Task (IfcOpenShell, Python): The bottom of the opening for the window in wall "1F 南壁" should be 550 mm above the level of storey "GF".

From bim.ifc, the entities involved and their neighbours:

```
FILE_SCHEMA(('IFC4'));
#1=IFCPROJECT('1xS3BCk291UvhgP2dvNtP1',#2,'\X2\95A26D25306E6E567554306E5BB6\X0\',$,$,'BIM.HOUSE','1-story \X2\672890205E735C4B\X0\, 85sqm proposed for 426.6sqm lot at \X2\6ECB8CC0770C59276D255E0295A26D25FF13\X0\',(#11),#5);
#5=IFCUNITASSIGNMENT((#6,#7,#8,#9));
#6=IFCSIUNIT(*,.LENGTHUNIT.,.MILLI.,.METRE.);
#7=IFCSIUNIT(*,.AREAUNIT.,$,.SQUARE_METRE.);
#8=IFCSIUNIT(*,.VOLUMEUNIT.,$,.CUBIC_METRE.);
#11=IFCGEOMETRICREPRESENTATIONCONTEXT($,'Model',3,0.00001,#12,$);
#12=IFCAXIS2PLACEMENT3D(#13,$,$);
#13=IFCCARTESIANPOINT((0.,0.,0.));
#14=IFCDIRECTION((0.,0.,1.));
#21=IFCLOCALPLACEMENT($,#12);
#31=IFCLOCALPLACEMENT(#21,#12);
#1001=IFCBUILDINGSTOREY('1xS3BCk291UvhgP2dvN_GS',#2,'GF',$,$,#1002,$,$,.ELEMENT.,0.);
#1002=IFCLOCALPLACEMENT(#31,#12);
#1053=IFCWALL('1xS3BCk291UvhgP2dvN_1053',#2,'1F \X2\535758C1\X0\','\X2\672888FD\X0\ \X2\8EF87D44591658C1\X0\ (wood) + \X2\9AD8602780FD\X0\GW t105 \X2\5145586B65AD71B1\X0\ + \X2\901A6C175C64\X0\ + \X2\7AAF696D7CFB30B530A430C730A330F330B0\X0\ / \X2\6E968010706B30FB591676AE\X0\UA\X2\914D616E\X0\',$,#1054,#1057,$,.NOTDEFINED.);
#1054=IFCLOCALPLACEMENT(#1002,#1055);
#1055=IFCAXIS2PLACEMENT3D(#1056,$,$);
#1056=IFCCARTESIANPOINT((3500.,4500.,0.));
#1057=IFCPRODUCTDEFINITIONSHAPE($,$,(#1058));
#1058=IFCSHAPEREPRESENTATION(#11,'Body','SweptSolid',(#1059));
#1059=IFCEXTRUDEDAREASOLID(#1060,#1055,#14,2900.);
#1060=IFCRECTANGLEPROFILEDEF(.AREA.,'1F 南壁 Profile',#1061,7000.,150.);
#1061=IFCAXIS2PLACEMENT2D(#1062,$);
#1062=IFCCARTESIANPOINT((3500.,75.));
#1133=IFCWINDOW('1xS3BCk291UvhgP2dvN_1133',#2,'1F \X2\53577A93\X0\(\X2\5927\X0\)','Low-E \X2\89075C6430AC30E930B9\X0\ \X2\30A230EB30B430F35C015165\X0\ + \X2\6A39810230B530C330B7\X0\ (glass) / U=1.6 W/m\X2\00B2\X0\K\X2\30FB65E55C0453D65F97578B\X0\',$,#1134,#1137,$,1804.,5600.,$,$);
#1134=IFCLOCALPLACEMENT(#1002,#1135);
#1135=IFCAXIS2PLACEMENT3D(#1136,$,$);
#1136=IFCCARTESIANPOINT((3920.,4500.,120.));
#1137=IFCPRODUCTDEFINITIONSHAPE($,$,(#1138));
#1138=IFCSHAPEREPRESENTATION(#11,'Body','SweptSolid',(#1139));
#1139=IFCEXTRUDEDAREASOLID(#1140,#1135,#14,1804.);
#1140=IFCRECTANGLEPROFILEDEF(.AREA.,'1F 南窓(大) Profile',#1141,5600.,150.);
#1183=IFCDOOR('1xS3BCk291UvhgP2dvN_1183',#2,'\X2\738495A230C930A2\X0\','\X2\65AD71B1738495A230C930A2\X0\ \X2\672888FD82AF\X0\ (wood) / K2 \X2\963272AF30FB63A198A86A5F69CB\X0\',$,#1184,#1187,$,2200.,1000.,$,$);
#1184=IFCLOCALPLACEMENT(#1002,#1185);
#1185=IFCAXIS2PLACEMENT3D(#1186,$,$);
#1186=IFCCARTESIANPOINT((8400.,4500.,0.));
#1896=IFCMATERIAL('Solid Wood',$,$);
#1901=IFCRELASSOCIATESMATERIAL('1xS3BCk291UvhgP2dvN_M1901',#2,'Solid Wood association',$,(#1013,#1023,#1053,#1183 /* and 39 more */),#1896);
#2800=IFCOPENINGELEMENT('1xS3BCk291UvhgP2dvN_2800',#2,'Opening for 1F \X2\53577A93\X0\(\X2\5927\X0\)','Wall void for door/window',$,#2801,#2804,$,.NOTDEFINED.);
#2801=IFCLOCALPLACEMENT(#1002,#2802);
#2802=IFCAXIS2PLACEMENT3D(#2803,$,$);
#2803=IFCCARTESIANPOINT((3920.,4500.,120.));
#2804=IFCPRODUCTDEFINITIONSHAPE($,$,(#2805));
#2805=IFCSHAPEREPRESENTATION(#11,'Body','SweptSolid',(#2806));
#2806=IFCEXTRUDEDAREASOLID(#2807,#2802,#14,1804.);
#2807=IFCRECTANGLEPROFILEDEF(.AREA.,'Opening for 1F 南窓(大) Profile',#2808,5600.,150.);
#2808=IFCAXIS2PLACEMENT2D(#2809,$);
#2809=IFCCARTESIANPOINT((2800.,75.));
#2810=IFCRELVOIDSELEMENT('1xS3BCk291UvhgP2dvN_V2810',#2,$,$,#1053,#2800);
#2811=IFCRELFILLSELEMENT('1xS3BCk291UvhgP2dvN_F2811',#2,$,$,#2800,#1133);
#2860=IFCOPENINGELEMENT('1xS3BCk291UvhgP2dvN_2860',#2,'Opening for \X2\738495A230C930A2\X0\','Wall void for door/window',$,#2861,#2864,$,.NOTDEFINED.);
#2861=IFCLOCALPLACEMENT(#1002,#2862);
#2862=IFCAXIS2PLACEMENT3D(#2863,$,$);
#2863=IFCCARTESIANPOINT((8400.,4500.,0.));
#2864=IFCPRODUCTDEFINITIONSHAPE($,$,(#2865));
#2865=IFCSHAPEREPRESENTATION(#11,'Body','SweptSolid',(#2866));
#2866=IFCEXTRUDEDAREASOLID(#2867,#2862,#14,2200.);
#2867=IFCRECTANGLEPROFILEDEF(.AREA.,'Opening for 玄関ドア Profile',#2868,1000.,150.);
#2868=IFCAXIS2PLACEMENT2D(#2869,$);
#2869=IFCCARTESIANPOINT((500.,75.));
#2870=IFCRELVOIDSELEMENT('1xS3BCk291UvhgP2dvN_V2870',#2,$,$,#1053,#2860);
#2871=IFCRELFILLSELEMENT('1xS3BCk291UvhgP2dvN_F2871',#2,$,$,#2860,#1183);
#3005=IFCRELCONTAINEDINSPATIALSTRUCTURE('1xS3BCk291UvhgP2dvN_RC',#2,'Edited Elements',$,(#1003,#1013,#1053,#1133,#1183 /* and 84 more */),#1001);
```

```python
import numpy as np
import ifcopenshell
import ifcopenshell.api.geometry
import ifcopenshell.geom
import ifcopenshell.util.element
import ifcopenshell.util.placement
import ifcopenshell.util.shape
import ifcopenshell.util.unit

model = ifcopenshell.open("bim.ifc")
unit_scale = ifcopenshell.util.unit.calculate_unit_scale(model)

window = model.by_guid("1xS3BCk291UvhgP2dvN_1133")
opening = window.FillsVoids[0].RelatingOpeningElement
storey = ifcopenshell.util.element.get_container(window, ifc_class="IfcBuildingStorey")
level = ifcopenshell.util.placement.get_local_placement(storey.ObjectPlacement)[2, 3]

# The opening's origin need not be at the sill, so measure its lowest point.
shape = ifcopenshell.geom.create_shape(ifcopenshell.geom.settings(), opening)
bottom = ifcopenshell.util.shape.get_shape_bottom_elevation(shape, shape.geometry) / unit_scale
dz = level + 550.0 - bottom

shift = np.array([0.0, 0.0, dz])
# The window is not placed relative to its opening, so move both.
for product in (opening, window):
    matrix = ifcopenshell.util.placement.get_local_placement(product.ObjectPlacement)
    matrix[:3, 3] += shift
    ifcopenshell.api.geometry.edit_object_placement(model, product=product, matrix=matrix, is_si=False)

print(f"moved by {dz * unit_scale:+.3f} m")

model.write("bim_updated.ifc")
```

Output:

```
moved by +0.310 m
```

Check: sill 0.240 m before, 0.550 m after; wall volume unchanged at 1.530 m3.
